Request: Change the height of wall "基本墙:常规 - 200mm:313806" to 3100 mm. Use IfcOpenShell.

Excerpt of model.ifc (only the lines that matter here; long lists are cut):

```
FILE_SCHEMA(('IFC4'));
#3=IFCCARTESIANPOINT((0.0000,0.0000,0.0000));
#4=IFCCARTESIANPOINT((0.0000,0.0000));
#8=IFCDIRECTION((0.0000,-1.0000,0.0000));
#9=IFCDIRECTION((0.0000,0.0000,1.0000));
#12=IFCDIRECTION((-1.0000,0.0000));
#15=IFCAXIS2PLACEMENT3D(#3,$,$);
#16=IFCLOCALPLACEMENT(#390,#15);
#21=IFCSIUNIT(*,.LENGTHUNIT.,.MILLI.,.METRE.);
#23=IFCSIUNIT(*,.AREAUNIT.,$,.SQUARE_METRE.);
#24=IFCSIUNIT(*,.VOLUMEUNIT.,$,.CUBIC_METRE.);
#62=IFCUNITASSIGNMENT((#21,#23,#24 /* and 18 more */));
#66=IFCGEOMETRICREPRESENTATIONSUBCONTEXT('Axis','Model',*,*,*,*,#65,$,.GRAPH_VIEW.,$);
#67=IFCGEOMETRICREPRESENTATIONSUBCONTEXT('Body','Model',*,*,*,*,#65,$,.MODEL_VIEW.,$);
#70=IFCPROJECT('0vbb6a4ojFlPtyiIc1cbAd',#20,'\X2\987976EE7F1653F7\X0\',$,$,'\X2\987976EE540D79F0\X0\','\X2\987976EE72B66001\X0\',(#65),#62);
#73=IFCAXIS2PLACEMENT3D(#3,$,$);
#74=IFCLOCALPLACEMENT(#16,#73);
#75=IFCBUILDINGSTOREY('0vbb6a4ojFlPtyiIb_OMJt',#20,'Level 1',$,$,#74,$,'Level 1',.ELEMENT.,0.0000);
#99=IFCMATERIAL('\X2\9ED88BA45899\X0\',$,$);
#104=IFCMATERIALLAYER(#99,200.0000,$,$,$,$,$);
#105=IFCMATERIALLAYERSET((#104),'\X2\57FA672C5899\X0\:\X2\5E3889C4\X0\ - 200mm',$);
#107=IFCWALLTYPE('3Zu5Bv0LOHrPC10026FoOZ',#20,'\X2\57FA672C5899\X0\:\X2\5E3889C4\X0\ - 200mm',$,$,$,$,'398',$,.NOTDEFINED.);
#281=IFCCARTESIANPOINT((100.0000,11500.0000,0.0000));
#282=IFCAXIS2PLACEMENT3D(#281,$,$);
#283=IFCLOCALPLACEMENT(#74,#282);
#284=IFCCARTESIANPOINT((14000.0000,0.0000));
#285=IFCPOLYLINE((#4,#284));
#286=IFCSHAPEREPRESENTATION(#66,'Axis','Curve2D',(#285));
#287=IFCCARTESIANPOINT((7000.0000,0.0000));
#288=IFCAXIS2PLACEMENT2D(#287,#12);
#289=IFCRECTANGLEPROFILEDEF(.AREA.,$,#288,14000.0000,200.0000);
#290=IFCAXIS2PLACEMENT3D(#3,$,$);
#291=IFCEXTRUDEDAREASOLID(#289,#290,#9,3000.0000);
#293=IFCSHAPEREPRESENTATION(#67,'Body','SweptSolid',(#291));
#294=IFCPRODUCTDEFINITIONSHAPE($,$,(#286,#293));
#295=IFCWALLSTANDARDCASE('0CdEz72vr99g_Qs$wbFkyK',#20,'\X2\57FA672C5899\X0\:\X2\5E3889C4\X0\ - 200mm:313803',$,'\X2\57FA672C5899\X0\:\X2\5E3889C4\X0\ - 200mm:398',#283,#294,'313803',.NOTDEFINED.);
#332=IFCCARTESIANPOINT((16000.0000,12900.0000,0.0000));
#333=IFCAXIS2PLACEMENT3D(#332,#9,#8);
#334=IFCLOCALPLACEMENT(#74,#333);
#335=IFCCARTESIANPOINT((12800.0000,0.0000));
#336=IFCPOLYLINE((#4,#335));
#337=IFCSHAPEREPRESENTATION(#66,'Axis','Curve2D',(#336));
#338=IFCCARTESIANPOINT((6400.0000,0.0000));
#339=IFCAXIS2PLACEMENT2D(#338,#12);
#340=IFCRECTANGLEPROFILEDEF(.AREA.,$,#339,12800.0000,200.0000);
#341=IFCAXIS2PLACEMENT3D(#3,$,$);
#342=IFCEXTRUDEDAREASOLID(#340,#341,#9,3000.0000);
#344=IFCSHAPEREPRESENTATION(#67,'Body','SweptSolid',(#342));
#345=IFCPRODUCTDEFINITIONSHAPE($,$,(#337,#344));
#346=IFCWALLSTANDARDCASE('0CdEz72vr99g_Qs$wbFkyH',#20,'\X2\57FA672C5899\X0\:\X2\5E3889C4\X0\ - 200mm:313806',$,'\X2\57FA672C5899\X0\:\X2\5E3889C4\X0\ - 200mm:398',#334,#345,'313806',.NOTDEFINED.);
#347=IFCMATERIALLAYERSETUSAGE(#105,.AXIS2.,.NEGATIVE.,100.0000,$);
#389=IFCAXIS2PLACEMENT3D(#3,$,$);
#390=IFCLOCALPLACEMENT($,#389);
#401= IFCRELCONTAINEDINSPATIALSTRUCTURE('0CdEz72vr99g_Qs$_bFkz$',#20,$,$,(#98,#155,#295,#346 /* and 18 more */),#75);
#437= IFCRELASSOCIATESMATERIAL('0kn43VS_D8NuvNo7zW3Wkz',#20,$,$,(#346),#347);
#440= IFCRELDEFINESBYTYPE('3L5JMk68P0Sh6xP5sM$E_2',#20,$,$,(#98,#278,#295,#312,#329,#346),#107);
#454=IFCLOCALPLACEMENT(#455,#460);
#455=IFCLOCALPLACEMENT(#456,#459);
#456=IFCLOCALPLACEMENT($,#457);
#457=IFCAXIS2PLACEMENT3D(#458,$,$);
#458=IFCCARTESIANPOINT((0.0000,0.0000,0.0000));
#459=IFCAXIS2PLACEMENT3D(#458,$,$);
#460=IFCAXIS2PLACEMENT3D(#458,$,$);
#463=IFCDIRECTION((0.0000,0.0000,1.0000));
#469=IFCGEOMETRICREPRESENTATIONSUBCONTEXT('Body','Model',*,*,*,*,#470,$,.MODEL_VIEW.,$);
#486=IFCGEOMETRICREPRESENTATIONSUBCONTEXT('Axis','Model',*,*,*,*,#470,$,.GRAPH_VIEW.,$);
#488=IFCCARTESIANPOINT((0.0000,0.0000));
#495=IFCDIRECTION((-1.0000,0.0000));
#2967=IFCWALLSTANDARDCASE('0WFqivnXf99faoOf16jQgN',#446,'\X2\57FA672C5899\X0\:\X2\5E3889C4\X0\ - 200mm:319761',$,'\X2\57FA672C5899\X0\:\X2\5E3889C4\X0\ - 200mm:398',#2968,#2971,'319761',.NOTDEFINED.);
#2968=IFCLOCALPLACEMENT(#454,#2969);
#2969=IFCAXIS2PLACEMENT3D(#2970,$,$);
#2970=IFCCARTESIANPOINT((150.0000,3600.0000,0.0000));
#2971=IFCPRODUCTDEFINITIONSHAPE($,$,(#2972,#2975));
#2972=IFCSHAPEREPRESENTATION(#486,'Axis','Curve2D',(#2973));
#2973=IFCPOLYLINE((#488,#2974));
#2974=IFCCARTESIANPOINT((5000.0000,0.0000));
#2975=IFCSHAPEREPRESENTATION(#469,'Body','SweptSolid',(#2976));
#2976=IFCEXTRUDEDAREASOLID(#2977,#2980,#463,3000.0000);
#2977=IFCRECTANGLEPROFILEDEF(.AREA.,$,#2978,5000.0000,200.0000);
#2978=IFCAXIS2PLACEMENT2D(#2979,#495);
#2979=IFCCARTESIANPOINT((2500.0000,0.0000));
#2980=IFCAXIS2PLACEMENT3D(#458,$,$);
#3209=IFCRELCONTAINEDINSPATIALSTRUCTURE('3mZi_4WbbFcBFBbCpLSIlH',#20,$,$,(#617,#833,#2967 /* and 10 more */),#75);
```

```python
import ifcopenshell
import ifcopenshell.geom
import ifcopenshell.util.representation
import ifcopenshell.util.shape
import ifcopenshell.util.unit

model = ifcopenshell.open("model.ifc")
unit_scale = ifcopenshell.util.unit.calculate_unit_scale(model)
settings = ifcopenshell.geom.settings()


def volume(element):
    """Net volume in cubic metres, openings subtracted."""
    shape = ifcopenshell.geom.create_shape(settings, element)
    return ifcopenshell.util.shape.get_volume(shape.geometry)


wall = model.by_id(346)
before = volume(wall)

body = ifcopenshell.util.representation.get_representation(wall, "Model", "Body")
solid = body.Items[0]
old_height = solid.Depth
solid.Depth = 3.1 / unit_scale
after = volume(wall)

print(f"height {old_height:g} -> {solid.Depth:g}, volume {before:.3f} -> {after:.3f} m3")

model.write("model_v2.ifc")
```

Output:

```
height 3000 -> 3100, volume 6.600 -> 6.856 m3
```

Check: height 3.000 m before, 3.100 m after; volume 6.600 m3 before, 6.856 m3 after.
